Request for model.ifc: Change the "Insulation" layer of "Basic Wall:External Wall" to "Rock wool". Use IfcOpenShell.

First a look at what the model holds.

```python
import ifcopenshell
import ifcopenshell.util.element

model = ifcopenshell.open("model.ifc")
print(model.schema)
for layer_set in model.by_type("IfcMaterialLayerSet"):
    if layer_set.LayerSetName == "Basic Wall:External Wall":
        for layer in layer_set.MaterialLayers:
            print(layer.id(), layer.Material and layer.Material.Name, layer.LayerThickness, sep=" | ")
        print(len(ifcopenshell.util.element.get_elements_by_material(model, layer_set)), "elements and types use it")
print(sorted(m.Name for m in model.by_type("IfcMaterial") if m.Name)[:60])
```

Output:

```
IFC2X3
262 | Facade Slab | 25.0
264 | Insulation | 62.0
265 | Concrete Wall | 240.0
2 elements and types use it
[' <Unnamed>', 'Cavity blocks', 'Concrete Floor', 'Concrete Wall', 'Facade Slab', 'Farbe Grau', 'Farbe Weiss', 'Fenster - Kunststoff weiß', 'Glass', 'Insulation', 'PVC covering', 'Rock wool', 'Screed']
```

```python
import ifcopenshell
import ifcopenshell.api.material

model = ifcopenshell.open("model.ifc")

layer_set = next(s for s in model.by_type("IfcMaterialLayerSet") if s.LayerSetName == "Basic Wall:External Wall")
layer = next(l for l in layer_set.MaterialLayers if l.Material and l.Material.Name == "Insulation")
material = next(m for m in model.by_type("IfcMaterial") if m.Name == "Rock wool")

# Point this one layer at the other material; renaming the old one would change it everywhere.
ifcopenshell.api.material.edit_layer(model, layer=layer, attributes={}, material=material)

print([l.Material.Name if l.Material else None for l in layer_set.MaterialLayers])

model.write("model-out.ifc")
```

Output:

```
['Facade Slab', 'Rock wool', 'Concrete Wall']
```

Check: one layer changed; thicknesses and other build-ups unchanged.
